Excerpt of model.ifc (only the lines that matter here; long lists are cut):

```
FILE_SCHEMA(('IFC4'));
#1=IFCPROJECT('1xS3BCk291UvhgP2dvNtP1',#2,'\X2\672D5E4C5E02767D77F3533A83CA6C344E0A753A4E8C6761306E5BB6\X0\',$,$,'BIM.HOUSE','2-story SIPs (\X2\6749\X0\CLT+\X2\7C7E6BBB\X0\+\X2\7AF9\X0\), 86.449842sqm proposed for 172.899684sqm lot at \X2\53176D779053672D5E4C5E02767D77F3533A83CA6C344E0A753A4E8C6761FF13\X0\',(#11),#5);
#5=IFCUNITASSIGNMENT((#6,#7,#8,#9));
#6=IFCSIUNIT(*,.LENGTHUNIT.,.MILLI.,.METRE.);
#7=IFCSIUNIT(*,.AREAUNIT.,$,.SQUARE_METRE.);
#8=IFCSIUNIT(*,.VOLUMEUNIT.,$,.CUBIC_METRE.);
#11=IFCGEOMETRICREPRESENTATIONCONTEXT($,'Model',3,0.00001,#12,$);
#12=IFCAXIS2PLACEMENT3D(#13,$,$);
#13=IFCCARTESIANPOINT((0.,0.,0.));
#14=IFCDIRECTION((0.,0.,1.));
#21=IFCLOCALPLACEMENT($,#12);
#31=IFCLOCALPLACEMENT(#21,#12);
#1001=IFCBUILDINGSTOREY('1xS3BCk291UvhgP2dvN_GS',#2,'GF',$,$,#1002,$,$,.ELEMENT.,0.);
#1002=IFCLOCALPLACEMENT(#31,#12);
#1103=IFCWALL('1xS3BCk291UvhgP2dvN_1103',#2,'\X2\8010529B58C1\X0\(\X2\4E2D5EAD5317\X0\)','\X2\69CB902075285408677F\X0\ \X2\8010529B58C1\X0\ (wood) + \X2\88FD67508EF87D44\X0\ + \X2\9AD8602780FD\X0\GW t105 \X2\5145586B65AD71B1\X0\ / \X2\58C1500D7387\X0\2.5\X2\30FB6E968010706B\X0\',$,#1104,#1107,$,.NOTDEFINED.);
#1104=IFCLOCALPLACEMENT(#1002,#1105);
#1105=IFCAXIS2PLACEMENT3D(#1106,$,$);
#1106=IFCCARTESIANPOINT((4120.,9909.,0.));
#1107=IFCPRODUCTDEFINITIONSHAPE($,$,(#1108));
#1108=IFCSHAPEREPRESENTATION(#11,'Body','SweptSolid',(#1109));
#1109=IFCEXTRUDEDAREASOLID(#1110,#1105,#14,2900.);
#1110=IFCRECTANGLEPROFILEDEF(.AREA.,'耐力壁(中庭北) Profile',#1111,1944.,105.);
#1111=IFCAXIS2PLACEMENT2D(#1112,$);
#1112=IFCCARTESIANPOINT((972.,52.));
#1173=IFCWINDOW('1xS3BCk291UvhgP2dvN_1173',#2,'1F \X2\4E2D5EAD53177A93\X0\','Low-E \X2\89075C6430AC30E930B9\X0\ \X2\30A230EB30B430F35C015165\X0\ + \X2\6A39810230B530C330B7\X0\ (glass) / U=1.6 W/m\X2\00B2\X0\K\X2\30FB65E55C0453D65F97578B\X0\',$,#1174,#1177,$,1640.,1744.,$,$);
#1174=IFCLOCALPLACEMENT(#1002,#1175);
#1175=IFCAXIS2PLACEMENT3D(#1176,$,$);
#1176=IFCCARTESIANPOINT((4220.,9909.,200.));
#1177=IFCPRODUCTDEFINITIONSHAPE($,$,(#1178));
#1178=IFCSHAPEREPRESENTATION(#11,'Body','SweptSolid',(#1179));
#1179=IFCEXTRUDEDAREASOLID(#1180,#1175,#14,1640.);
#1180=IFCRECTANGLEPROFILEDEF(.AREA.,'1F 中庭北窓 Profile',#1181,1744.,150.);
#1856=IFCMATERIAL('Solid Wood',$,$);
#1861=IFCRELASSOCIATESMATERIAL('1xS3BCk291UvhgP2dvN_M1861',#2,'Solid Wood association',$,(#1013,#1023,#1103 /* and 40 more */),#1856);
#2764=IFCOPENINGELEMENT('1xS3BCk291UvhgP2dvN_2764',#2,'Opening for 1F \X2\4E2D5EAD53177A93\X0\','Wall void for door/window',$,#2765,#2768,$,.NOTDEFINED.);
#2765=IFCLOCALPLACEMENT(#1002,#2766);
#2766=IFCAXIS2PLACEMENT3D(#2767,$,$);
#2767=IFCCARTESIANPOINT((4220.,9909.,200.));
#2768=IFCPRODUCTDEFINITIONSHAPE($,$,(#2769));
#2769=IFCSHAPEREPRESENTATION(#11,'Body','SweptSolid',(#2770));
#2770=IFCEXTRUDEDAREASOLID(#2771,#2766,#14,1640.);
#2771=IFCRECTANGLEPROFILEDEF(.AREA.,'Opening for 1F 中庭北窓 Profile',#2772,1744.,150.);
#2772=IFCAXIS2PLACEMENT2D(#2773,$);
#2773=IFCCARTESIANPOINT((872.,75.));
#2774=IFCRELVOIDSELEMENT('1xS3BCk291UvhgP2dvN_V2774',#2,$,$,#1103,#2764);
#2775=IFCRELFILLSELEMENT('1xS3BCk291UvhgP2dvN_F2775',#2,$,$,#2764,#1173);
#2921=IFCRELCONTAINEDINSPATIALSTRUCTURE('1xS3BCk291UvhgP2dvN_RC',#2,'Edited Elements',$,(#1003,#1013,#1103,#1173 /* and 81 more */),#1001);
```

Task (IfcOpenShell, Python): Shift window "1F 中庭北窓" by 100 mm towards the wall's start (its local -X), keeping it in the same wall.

```python
import ifcopenshell
import ifcopenshell.api.geometry
import ifcopenshell.util.placement
import ifcopenshell.util.unit

model = ifcopenshell.open("model.ifc")
unit_scale = ifcopenshell.util.unit.calculate_unit_scale(model)

window = model.by_guid("1xS3BCk291UvhgP2dvN_1173")
opening = window.FillsVoids[0].RelatingOpeningElement
wall = opening.VoidsElements[0].RelatingBuildingElement

wall_matrix = ifcopenshell.util.placement.get_local_placement(wall.ObjectPlacement)
shift = wall_matrix[:3, 0] * -0.1 / unit_scale
before = ifcopenshell.util.placement.get_local_placement(window.ObjectPlacement)[:3, 3].copy()

# The window is not placed relative to its opening, so move both.
for product in (opening, window):
    matrix = ifcopenshell.util.placement.get_local_placement(product.ObjectPlacement)
    matrix[:3, 3] += shift
    ifcopenshell.api.geometry.edit_object_placement(model, product=product, matrix=matrix, is_si=False)

after = ifcopenshell.util.placement.get_local_placement(window.ObjectPlacement)[:3, 3]
print("window moved by", (after - before).round(3) + 0.0)

model.write("model_edited.ifc")
```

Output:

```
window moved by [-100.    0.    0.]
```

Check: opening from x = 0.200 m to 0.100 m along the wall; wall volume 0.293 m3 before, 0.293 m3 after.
